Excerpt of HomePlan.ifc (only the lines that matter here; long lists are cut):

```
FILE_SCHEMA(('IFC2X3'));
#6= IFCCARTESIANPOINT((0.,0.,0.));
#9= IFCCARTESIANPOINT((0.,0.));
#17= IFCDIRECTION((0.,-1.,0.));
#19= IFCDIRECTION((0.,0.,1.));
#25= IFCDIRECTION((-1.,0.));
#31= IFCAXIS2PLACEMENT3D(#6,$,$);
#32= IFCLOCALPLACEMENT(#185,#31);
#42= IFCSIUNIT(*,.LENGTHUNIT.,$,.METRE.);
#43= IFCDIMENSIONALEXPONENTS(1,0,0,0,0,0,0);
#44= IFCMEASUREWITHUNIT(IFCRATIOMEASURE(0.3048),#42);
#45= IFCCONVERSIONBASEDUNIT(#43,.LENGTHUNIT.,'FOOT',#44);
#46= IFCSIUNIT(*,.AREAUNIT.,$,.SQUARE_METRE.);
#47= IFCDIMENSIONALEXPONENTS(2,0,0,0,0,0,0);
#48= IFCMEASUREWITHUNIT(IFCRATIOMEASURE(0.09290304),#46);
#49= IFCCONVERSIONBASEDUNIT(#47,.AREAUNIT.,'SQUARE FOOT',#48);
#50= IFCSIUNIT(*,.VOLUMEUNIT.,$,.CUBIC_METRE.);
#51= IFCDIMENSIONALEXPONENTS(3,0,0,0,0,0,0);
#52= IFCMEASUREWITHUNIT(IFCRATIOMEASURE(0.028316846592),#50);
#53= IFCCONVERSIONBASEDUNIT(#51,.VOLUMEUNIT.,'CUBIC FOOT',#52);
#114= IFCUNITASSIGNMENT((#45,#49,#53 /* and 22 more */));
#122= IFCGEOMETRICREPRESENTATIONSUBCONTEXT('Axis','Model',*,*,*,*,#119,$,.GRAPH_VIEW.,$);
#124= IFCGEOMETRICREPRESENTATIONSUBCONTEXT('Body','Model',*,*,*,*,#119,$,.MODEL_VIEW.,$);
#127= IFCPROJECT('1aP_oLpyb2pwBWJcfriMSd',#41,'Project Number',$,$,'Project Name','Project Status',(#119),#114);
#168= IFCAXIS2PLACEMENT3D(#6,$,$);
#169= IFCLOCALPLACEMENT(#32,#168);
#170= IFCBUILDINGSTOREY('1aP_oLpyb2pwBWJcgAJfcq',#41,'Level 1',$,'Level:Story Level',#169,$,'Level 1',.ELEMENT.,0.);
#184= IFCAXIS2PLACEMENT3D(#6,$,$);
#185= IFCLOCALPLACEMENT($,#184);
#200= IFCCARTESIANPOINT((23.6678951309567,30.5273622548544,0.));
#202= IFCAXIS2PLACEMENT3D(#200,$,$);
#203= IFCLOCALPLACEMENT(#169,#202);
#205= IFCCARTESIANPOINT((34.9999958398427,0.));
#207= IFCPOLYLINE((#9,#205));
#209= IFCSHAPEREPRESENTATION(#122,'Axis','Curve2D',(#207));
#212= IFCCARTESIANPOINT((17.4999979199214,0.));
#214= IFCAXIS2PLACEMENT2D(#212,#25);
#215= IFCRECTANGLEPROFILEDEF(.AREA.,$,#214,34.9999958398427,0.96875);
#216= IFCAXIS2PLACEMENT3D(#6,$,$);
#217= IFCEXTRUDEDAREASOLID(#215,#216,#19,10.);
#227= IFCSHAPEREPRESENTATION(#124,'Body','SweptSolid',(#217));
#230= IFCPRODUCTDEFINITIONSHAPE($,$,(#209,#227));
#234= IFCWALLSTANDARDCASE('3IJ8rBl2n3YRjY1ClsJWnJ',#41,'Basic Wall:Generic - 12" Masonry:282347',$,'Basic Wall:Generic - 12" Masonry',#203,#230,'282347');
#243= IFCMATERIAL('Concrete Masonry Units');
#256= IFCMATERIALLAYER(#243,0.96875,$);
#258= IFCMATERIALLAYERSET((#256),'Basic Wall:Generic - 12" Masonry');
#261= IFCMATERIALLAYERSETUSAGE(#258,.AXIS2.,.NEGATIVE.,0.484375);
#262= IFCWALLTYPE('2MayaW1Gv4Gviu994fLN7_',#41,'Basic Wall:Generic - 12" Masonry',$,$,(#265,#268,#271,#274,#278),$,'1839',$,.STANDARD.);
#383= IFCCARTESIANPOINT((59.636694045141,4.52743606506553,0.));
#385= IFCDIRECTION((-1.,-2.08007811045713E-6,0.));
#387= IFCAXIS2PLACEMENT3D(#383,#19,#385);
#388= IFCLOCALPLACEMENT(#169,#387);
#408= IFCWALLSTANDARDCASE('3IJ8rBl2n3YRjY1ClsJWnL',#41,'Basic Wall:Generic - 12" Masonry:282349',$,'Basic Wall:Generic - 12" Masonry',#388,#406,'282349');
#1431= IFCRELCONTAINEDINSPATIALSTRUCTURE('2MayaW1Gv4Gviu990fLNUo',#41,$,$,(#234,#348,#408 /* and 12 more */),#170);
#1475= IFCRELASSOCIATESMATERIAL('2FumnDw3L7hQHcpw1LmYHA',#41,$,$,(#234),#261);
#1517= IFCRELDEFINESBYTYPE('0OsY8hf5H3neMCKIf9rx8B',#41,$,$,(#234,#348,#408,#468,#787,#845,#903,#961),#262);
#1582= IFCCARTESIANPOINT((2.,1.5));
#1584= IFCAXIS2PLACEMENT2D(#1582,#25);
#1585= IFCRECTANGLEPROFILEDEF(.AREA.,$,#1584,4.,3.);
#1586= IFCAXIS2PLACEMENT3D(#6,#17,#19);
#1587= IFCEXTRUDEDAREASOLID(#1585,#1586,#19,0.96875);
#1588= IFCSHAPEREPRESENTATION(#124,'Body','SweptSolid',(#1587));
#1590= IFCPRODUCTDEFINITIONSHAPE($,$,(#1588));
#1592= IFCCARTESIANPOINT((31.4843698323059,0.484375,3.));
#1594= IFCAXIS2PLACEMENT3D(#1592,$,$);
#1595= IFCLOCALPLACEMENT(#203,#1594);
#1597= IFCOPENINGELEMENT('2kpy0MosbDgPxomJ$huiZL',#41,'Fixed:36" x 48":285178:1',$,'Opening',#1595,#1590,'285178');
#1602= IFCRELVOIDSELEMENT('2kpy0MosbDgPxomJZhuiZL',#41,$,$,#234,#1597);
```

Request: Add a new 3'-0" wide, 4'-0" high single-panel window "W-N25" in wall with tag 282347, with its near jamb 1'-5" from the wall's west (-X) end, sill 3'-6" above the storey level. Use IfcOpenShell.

```python
import numpy as np
import ifcopenshell
import ifcopenshell.api.feature
import ifcopenshell.api.geometry
import ifcopenshell.api.root
import ifcopenshell.api.spatial
import ifcopenshell.api.type
import ifcopenshell.geom
import ifcopenshell.util.element
import ifcopenshell.util.placement
import ifcopenshell.util.representation
import ifcopenshell.util.shape
import ifcopenshell.util.unit

model = ifcopenshell.open("HomePlan.ifc")
unit_scale = ifcopenshell.util.unit.calculate_unit_scale(model)
settings = ifcopenshell.geom.settings()


def volume(element):
    """Net volume in cubic metres, openings subtracted."""
    shape = ifcopenshell.geom.create_shape(settings, element)
    return ifcopenshell.util.shape.get_volume(shape.geometry)


wall = model.by_guid("3IJ8rBl2n3YRjY1ClsJWnJ")
storey = ifcopenshell.util.element.get_container(wall, ifc_class="IfcBuildingStorey")
context = ifcopenshell.util.representation.get_context(model, "Model", "Body", "MODEL_VIEW")
before = volume(wall)

width, height, from_end, sill = 0.9144, 1.2192, 0.4318, 1.0668  # metres

# The wall runs along its own X axis, and the end named is its -X end.
wall_shape = ifcopenshell.geom.create_shape(settings, wall)
x, y, z = ifcopenshell.util.shape.get_vertices(wall_shape.geometry).T
start = x.min() + from_end
face, thickness = float(y.min()), float(y.max() - y.min())
wall_matrix = ifcopenshell.util.placement.get_local_placement(wall.ObjectPlacement)
level = ifcopenshell.util.placement.get_local_placement(storey.ObjectPlacement)[2, 3]


def in_wall(x, y):
    """Placement at x, y metres in the wall's axes, at sill height."""
    matrix = wall_matrix.copy()
    matrix[:, 3] = wall_matrix @ np.array([x / unit_scale, y / unit_scale, 0.0, 1.0])
    matrix[2, 3] = level + sill / unit_scale
    return matrix


# Opening: a box that overshoots both wall faces by 50 mm.
opening = ifcopenshell.api.root.create_entity(model, ifc_class="IfcOpeningElement")
box = ifcopenshell.api.geometry.add_wall_representation(
    model, context=context, length=width, height=height, thickness=thickness + 0.1
)
ifcopenshell.api.geometry.assign_representation(model, product=opening, representation=box)
ifcopenshell.api.geometry.edit_object_placement(model, product=opening, matrix=in_wall(start, face - 0.05), is_si=False)
ifcopenshell.api.feature.add_feature(model, feature=opening, element=wall)

window = ifcopenshell.api.root.create_entity(model, ifc_class="IfcWindow", name="W-N25")
window.OverallWidth, window.OverallHeight = width / unit_scale, height / unit_scale
body = ifcopenshell.api.geometry.add_window_representation(
    model,
    context=context,
    overall_width=window.OverallWidth,
    overall_height=window.OverallHeight,
    partition_type="SINGLE_PANEL",
)
ifcopenshell.api.geometry.assign_representation(model, product=window, representation=body)
ifcopenshell.api.spatial.assign_container(model, products=[window], relating_structure=storey)
fills = ifcopenshell.api.feature.add_filling(model, opening=opening, element=window)
fills.OwnerHistory = window.OwnerHistory  # required in IFC2X3

# IFC2X3 keeps the operation on the window style.
style = ifcopenshell.api.root.create_entity(model, ifc_class="IfcWindowStyle", name="W-N25")
style.OperationType, style.ConstructionType = "SINGLE_PANEL", "NOTDEFINED"
style.ParameterTakesPrecedence = style.Sizeable = False
ifcopenshell.api.type.assign_type(model, related_objects=[window], relating_type=style)

# Centre the window in the wall's thickness.
ifcopenshell.api.geometry.edit_object_placement(model, product=window, matrix=in_wall(start, face), is_si=False)
window_shape = ifcopenshell.geom.create_shape(settings, window)
depth = ifcopenshell.util.shape.get_vertices(window_shape.geometry)[:, 1]
offset = face + thickness / 2 - (depth.min() + depth.max()) / 2
ifcopenshell.api.geometry.edit_object_placement(model, product=window, matrix=in_wall(start, offset), is_si=False)

after = volume(wall)

print(f"wall volume {before:.3f} -> {after:.3f} m3")

model.write("HomePlan_edited.ifc")
```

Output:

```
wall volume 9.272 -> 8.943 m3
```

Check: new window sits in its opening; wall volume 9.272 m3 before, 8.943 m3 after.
